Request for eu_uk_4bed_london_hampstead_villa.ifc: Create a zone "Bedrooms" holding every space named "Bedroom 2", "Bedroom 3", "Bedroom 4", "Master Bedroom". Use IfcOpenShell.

First a look at what the model holds.

```python
import ifcopenshell

model = ifcopenshell.open("eu_uk_4bed_london_hampstead_villa.ifc")
print(model.schema)
seen = {}
for space in model.by_type("IfcSpace"):
    seen[space.LongName] = seen.get(space.LongName, 0) + 1
for name, count in sorted(seen.items(), key=str):
    print(count, "x", name)
print("zones:", [z.Name for z in model.by_type("IfcZone")][:20])
```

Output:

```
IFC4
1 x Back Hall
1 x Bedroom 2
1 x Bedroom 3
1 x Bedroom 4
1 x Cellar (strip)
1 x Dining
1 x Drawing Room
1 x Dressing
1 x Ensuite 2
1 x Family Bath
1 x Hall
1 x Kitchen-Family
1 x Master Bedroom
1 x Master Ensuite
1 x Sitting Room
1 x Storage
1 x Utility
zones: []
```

```python
import ifcopenshell
import ifcopenshell.api.group
import ifcopenshell.api.root

model = ifcopenshell.open("eu_uk_4bed_london_hampstead_villa.ifc")

names = {"Bedroom 2", "Bedroom 3", "Bedroom 4", "Master Bedroom"}
spaces = [s for s in model.by_type("IfcSpace") if s.LongName in names]

zone = ifcopenshell.api.root.create_entity(model, ifc_class="IfcZone", name="Bedrooms")
ifcopenshell.api.group.assign_group(model, products=spaces, group=zone)
print(len(spaces), "spaces in", zone.Name)

model.write("eu_uk_4bed_london_hampstead_villa_edited.ifc")
```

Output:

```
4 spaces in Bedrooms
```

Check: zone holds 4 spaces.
